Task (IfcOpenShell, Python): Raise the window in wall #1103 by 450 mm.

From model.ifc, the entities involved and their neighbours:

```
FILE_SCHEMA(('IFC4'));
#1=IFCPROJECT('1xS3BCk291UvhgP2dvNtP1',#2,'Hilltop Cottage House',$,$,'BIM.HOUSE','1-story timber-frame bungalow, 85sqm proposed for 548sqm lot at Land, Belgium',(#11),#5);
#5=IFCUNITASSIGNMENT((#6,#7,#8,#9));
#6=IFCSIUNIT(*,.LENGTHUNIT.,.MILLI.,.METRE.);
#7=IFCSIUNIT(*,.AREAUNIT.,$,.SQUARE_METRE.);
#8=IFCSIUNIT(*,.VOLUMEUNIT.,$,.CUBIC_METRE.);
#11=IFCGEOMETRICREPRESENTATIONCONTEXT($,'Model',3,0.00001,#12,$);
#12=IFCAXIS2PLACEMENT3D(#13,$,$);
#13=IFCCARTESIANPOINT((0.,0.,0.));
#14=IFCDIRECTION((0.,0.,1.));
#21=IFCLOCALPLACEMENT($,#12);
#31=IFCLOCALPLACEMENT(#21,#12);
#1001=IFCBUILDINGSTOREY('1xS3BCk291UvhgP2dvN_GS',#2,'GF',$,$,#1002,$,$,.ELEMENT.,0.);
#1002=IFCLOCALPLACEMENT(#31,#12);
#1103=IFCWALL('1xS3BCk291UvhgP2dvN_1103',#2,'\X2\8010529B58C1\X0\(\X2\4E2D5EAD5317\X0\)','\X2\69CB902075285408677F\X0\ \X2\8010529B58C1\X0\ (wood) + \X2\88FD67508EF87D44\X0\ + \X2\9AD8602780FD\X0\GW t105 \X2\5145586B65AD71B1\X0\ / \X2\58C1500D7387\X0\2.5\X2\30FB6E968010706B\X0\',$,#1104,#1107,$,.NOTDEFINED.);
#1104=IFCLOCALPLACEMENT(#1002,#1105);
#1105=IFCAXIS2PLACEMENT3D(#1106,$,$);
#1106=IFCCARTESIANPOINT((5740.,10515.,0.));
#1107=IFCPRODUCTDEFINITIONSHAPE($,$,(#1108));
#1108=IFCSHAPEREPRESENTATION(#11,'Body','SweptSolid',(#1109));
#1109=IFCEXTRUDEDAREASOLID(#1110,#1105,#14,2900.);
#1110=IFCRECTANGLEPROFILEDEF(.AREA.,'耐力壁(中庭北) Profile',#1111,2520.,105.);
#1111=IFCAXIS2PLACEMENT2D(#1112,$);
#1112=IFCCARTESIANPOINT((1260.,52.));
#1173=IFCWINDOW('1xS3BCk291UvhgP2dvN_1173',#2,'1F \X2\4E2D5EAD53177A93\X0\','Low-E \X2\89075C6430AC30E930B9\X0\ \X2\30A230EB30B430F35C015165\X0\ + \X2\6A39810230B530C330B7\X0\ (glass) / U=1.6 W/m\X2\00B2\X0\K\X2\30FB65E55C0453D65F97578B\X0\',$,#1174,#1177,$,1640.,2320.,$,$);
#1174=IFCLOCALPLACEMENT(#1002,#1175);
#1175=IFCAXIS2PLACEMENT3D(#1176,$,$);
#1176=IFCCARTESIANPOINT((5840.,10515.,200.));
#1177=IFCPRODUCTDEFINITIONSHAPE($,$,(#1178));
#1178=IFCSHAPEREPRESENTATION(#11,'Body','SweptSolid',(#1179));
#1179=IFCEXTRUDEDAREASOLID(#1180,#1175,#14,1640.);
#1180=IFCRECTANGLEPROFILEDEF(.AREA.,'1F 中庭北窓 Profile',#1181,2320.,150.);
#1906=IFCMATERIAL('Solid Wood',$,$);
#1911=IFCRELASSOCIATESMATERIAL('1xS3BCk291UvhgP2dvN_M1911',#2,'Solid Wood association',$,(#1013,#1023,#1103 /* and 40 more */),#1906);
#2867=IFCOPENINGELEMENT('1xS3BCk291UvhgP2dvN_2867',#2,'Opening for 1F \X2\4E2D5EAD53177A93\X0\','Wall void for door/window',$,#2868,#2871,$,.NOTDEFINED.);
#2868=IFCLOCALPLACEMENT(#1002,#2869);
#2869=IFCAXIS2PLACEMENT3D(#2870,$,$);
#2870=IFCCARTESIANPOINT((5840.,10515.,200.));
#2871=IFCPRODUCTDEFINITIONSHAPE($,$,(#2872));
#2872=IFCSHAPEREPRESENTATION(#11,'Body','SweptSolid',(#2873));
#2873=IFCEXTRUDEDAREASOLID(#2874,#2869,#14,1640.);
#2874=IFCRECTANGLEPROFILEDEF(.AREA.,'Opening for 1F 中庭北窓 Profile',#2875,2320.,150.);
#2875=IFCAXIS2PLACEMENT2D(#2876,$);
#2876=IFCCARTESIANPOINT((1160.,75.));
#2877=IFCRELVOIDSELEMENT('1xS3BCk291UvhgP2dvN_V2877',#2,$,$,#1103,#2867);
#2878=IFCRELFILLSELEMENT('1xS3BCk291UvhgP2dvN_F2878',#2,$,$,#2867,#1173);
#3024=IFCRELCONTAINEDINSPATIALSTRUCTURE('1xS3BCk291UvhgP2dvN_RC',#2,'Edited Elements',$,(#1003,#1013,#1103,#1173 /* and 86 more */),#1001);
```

```python
import numpy as np
import ifcopenshell
import ifcopenshell.api.geometry
import ifcopenshell.util.placement
import ifcopenshell.util.unit

model = ifcopenshell.open("model.ifc")
unit_scale = ifcopenshell.util.unit.calculate_unit_scale(model)

window = model.by_guid("1xS3BCk291UvhgP2dvN_1173")
opening = window.FillsVoids[0].RelatingOpeningElement
dz = 450.0

shift = np.array([0.0, 0.0, dz])
# The window is not placed relative to its opening, so move both.
for product in (opening, window):
    matrix = ifcopenshell.util.placement.get_local_placement(product.ObjectPlacement)
    matrix[:3, 3] += shift
    ifcopenshell.api.geometry.edit_object_placement(model, product=product, matrix=matrix, is_si=False)

print(f"moved by {dz * unit_scale:+.3f} m")

model.write("model-out.ifc")
```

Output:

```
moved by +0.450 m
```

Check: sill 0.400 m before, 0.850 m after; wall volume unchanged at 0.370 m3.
